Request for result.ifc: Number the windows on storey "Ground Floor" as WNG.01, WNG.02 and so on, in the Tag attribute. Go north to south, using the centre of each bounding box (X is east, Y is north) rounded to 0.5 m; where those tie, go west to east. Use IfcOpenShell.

First a look at what the model holds.

```python
import ifcopenshell
import ifcopenshell.util.element
import ifcopenshell.util.placement

model = ifcopenshell.open("result.ifc")
print(model.schema)
storey = next(s for s in model.by_type("IfcBuildingStorey") if s.Name == "Ground Floor")
windows = [e for e in ifcopenshell.util.element.get_decomposition(storey) if e.is_a("IfcWindow")]
for e in sorted(windows, key=lambda e: e.id()):
    origin = ifcopenshell.util.placement.get_local_placement(e.ObjectPlacement)[:3, 3]
    print(e.id(), e.Tag, e.Name, origin.round(2) + 0.0, sep=" | ")
```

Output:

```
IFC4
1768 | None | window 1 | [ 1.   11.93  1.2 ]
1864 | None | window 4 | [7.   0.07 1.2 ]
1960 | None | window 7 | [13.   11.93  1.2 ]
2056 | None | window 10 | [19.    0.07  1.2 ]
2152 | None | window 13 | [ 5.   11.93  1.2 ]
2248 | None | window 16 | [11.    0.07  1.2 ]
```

```python
import ifcopenshell
import ifcopenshell.geom
import ifcopenshell.util.element
import ifcopenshell.util.shape

model = ifcopenshell.open("result.ifc")
settings = ifcopenshell.geom.settings()
settings.set("use-world-coords", True)


def centre(element):
    shape = ifcopenshell.geom.create_shape(settings, element)
    return ifcopenshell.util.shape.get_bbox_centroid(shape.geometry)


storey = next(s for s in model.by_type("IfcBuildingStorey") if s.Name == "Ground Floor")
windows = [e for e in ifcopenshell.util.element.get_decomposition(storey) if e.is_a("IfcWindow")]

# Insertion points can sit at a corner or the storey origin, so sort by the geometry (in metres).
centres = {e: centre(e) for e in windows}
windows.sort(key=lambda e: (-round(centres[e][1] / 0.5), centres[e][0]))

for i, e in enumerate(windows, start=1):
    number = f"WNG.{i:02d}"
    e.Tag = number
    print(e.id(), number)

model.write("result_updated.ifc")
```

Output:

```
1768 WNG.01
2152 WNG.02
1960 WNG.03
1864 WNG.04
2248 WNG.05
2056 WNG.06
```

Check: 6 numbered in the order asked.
